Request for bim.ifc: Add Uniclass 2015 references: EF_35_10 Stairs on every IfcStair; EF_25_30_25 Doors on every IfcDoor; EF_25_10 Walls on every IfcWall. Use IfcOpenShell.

First a look at what the model holds.

```python
import ifcopenshell

model = ifcopenshell.open("bim.ifc")
print(model.schema)
print("classifications:", [c.Name for c in model.by_type("IfcClassification")])
for ifc_class in ("IfcDoor", "IfcRoof", "IfcStair", "IfcWall", "IfcWindow"):
    print(ifc_class, len(model.by_type(ifc_class)))
```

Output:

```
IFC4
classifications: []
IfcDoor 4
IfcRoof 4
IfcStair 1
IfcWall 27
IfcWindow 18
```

```python
import ifcopenshell
import ifcopenshell.api.classification

model = ifcopenshell.open("bim.ifc")

system = ifcopenshell.api.classification.add_classification(model, classification="Uniclass 2015")

codes = {
    "IfcStair": ("EF_35_10", "Stairs"),
    "IfcDoor": ("EF_25_30_25", "Doors"),
    "IfcWall": ("EF_25_10", "Walls"),
}
for ifc_class, (code, name) in codes.items():
    products = model.by_type(ifc_class)
    ifcopenshell.api.classification.add_reference(
        model, products=products, classification=system, identification=code, name=name
    )
    print(code, len(products))

model.write("bim_updated.ifc")
```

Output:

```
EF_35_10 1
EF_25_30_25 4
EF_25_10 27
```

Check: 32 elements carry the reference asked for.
